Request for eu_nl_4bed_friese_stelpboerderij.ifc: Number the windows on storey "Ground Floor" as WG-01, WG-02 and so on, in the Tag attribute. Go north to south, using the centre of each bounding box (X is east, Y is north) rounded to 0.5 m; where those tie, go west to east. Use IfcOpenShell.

First a look at what the model holds.

```python
import ifcopenshell
import ifcopenshell.util.element
import ifcopenshell.util.placement

model = ifcopenshell.open("eu_nl_4bed_friese_stelpboerderij.ifc")
print(model.schema)
storey = next(s for s in model.by_type("IfcBuildingStorey") if s.Name == "Ground Floor")
windows = [e for e in ifcopenshell.util.element.get_decomposition(storey) if e.is_a("IfcWindow")]
for e in sorted(windows, key=lambda e: e.id()):
    origin = ifcopenshell.util.placement.get_local_placement(e.ObjectPlacement)[:3, 3]
    print(e.id(), e.Tag, e.Name, origin.round(2) + 0.0, sep=" | ")
```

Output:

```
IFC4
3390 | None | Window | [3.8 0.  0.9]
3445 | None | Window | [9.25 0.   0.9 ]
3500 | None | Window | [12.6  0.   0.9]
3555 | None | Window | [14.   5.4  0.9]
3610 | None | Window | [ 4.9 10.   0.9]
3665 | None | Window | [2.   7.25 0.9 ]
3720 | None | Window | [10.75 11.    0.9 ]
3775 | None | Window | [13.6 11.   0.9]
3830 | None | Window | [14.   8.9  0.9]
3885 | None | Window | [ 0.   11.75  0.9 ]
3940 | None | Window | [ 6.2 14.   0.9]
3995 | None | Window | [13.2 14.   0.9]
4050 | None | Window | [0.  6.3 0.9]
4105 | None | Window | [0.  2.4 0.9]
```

```python
import ifcopenshell
import ifcopenshell.geom
import ifcopenshell.util.element
import ifcopenshell.util.shape

model = ifcopenshell.open("eu_nl_4bed_friese_stelpboerderij.ifc")
settings = ifcopenshell.geom.settings()
settings.set("use-world-coords", True)


def centre(element):
    shape = ifcopenshell.geom.create_shape(settings, element)
    return ifcopenshell.util.shape.get_bbox_centroid(shape.geometry)


storey = next(s for s in model.by_type("IfcBuildingStorey") if s.Name == "Ground Floor")
windows = [e for e in ifcopenshell.util.element.get_decomposition(storey) if e.is_a("IfcWindow")]

# Insertion points can sit at a corner or the storey origin, so sort by the geometry (in metres).
centres = {e: centre(e) for e in windows}
windows.sort(key=lambda e: (-round(centres[e][1] / 0.5), centres[e][0]))

for i, e in enumerate(windows, start=1):
    number = f"WG-{i:02d}"
    e.Tag = number
    print(e.id(), number)

model.write("eu_nl_4bed_friese_stelpboerderij_updated.ifc")
```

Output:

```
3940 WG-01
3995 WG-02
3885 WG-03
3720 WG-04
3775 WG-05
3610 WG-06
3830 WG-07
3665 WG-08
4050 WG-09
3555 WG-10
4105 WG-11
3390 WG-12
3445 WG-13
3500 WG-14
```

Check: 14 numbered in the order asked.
